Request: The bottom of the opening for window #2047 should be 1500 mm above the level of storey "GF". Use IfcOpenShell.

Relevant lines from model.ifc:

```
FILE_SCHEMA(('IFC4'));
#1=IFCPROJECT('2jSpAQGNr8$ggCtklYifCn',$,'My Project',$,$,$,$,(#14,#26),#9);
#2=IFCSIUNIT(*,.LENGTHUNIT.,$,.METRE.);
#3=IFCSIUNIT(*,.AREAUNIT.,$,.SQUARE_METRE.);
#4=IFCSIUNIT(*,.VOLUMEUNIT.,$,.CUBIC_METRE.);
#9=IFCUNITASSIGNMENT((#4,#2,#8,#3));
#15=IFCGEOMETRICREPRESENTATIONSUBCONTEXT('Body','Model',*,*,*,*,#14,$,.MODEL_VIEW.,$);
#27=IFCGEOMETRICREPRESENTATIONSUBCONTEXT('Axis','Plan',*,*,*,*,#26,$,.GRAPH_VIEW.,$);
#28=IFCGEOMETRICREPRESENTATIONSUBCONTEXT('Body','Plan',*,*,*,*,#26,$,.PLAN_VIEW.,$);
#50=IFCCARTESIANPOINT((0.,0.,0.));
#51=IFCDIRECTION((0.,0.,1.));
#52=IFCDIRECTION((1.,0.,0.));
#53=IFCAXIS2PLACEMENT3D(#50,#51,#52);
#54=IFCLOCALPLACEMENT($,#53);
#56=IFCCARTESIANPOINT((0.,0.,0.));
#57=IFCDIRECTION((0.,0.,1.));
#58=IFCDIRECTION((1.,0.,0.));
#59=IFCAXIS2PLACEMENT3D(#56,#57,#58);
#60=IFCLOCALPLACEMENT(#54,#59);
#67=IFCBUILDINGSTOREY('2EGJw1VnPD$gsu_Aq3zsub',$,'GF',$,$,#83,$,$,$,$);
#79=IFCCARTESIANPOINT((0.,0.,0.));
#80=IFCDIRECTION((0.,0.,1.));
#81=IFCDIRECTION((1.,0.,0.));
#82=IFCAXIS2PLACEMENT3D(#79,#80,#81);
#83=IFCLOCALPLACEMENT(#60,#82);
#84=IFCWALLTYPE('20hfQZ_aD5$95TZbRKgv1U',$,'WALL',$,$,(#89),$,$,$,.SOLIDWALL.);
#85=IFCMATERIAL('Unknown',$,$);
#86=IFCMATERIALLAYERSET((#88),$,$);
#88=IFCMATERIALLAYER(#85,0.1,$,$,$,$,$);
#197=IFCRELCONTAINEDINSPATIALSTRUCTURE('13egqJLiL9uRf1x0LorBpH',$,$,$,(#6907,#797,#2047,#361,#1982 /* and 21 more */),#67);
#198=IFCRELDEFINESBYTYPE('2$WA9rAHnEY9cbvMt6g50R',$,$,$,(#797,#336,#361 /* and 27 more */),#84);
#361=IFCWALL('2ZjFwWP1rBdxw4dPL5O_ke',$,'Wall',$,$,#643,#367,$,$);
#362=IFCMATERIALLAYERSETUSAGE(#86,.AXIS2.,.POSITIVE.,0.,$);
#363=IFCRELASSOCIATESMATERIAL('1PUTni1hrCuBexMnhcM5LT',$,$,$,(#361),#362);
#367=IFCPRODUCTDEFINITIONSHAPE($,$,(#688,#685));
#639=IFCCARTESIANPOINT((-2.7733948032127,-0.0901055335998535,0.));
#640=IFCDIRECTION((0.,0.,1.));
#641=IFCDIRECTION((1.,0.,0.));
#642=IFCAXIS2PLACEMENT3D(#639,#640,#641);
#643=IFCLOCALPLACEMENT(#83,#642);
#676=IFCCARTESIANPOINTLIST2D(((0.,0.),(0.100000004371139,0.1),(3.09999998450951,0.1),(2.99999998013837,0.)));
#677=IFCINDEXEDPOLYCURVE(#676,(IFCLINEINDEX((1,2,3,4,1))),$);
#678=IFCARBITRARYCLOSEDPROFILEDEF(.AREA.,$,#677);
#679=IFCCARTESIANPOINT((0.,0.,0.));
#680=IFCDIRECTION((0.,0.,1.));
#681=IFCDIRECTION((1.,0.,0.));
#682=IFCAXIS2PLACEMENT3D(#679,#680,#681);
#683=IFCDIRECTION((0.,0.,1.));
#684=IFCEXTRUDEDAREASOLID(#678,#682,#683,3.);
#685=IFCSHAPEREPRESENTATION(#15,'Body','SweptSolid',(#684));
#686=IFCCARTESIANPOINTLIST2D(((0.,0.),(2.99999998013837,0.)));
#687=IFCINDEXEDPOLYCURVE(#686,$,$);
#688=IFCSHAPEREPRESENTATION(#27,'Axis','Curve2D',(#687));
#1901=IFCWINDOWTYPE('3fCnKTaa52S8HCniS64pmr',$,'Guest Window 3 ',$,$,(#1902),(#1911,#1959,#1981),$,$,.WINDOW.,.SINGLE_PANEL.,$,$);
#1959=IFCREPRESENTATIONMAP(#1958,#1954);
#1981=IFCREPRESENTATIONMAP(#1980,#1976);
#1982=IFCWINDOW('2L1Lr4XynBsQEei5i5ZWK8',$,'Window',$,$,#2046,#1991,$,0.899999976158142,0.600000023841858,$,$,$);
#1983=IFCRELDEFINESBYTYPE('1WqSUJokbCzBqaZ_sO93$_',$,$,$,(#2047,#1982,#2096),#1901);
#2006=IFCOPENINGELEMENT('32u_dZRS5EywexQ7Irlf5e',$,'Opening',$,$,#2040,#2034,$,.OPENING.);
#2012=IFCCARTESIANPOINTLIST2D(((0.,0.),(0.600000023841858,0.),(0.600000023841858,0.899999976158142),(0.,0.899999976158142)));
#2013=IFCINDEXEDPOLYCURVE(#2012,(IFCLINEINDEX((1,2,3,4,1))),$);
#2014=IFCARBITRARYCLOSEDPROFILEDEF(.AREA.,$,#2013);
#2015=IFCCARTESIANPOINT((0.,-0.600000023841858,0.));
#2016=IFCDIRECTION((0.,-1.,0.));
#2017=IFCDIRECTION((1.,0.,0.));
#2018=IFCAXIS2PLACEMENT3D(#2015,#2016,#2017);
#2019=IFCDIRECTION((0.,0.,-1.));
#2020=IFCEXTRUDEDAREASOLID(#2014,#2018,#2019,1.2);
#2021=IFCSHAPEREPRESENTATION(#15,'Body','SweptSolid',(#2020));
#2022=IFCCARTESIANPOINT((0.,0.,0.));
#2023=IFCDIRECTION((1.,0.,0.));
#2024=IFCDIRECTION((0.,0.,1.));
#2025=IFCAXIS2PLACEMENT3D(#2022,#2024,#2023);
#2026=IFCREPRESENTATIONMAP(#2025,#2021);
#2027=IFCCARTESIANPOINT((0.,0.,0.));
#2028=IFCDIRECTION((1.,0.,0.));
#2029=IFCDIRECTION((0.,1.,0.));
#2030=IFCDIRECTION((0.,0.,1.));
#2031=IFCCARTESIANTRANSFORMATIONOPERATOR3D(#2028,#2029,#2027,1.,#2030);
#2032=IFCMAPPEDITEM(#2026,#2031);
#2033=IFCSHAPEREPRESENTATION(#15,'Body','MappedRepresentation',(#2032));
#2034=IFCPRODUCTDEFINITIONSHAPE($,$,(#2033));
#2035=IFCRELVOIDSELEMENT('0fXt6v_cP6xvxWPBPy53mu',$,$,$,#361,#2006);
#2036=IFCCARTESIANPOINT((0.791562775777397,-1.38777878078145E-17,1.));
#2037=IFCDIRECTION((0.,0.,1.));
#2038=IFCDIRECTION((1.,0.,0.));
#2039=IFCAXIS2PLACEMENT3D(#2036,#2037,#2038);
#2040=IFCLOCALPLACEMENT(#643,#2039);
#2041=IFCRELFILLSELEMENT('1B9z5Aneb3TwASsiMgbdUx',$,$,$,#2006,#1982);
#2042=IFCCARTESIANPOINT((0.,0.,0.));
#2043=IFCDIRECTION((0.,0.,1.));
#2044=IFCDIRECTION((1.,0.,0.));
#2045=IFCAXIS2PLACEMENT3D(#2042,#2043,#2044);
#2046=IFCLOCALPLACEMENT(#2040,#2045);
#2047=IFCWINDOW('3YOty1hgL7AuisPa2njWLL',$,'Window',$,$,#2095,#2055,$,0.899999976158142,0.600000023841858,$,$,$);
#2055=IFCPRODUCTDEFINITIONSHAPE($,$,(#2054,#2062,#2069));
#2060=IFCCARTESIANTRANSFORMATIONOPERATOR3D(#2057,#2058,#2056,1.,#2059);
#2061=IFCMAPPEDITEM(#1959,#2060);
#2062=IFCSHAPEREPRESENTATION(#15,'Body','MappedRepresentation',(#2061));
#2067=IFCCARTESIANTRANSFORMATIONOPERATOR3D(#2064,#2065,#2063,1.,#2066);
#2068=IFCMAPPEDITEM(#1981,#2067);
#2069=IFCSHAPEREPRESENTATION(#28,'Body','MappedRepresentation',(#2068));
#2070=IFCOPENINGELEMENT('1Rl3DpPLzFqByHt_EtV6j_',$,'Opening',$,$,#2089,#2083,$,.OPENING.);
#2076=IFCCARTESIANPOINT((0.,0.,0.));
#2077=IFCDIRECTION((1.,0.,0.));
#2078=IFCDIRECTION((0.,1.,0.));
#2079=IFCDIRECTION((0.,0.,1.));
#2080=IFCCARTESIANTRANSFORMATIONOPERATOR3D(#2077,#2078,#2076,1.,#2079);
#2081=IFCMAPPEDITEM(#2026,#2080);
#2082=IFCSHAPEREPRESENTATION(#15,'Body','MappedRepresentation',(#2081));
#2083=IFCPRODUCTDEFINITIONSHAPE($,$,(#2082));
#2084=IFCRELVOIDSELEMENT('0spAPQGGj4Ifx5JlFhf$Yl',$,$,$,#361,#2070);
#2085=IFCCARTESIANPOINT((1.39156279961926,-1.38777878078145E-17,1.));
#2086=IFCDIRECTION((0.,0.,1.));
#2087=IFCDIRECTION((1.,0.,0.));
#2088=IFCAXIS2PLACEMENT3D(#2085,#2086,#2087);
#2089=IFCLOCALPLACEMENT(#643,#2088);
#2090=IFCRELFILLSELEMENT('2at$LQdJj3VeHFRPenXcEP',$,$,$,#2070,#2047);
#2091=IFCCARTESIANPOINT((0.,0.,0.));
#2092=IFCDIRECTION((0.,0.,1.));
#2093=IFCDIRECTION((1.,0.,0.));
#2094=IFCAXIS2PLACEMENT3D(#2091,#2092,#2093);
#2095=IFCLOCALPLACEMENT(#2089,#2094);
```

```python
import numpy as np
import ifcopenshell
import ifcopenshell.api.geometry
import ifcopenshell.geom
import ifcopenshell.util.element
import ifcopenshell.util.placement
import ifcopenshell.util.shape
import ifcopenshell.util.unit

model = ifcopenshell.open("model.ifc")
unit_scale = ifcopenshell.util.unit.calculate_unit_scale(model)

window = model.by_guid("3YOty1hgL7AuisPa2njWLL")
opening = window.FillsVoids[0].RelatingOpeningElement
storey = ifcopenshell.util.element.get_container(window, ifc_class="IfcBuildingStorey")
level = ifcopenshell.util.placement.get_local_placement(storey.ObjectPlacement)[2, 3]

# The opening's origin need not be at the sill, so measure its lowest point.
shape = ifcopenshell.geom.create_shape(ifcopenshell.geom.settings(), opening)
bottom = ifcopenshell.util.shape.get_shape_bottom_elevation(shape, shape.geometry) / unit_scale
dz = level + 1.5 / unit_scale - bottom

shift = np.array([0.0, 0.0, dz])
# The window is placed relative to its opening, so it follows when the opening moves.
matrix = ifcopenshell.util.placement.get_local_placement(opening.ObjectPlacement)
matrix[:3, 3] += shift
ifcopenshell.api.geometry.edit_object_placement(
    model, product=opening, matrix=matrix, is_si=False, should_transform_children=True
)

print(f"moved by {dz * unit_scale:+.3f} m")

model.write("model_v2.ifc")
```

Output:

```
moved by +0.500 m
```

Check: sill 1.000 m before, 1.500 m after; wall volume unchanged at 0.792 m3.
